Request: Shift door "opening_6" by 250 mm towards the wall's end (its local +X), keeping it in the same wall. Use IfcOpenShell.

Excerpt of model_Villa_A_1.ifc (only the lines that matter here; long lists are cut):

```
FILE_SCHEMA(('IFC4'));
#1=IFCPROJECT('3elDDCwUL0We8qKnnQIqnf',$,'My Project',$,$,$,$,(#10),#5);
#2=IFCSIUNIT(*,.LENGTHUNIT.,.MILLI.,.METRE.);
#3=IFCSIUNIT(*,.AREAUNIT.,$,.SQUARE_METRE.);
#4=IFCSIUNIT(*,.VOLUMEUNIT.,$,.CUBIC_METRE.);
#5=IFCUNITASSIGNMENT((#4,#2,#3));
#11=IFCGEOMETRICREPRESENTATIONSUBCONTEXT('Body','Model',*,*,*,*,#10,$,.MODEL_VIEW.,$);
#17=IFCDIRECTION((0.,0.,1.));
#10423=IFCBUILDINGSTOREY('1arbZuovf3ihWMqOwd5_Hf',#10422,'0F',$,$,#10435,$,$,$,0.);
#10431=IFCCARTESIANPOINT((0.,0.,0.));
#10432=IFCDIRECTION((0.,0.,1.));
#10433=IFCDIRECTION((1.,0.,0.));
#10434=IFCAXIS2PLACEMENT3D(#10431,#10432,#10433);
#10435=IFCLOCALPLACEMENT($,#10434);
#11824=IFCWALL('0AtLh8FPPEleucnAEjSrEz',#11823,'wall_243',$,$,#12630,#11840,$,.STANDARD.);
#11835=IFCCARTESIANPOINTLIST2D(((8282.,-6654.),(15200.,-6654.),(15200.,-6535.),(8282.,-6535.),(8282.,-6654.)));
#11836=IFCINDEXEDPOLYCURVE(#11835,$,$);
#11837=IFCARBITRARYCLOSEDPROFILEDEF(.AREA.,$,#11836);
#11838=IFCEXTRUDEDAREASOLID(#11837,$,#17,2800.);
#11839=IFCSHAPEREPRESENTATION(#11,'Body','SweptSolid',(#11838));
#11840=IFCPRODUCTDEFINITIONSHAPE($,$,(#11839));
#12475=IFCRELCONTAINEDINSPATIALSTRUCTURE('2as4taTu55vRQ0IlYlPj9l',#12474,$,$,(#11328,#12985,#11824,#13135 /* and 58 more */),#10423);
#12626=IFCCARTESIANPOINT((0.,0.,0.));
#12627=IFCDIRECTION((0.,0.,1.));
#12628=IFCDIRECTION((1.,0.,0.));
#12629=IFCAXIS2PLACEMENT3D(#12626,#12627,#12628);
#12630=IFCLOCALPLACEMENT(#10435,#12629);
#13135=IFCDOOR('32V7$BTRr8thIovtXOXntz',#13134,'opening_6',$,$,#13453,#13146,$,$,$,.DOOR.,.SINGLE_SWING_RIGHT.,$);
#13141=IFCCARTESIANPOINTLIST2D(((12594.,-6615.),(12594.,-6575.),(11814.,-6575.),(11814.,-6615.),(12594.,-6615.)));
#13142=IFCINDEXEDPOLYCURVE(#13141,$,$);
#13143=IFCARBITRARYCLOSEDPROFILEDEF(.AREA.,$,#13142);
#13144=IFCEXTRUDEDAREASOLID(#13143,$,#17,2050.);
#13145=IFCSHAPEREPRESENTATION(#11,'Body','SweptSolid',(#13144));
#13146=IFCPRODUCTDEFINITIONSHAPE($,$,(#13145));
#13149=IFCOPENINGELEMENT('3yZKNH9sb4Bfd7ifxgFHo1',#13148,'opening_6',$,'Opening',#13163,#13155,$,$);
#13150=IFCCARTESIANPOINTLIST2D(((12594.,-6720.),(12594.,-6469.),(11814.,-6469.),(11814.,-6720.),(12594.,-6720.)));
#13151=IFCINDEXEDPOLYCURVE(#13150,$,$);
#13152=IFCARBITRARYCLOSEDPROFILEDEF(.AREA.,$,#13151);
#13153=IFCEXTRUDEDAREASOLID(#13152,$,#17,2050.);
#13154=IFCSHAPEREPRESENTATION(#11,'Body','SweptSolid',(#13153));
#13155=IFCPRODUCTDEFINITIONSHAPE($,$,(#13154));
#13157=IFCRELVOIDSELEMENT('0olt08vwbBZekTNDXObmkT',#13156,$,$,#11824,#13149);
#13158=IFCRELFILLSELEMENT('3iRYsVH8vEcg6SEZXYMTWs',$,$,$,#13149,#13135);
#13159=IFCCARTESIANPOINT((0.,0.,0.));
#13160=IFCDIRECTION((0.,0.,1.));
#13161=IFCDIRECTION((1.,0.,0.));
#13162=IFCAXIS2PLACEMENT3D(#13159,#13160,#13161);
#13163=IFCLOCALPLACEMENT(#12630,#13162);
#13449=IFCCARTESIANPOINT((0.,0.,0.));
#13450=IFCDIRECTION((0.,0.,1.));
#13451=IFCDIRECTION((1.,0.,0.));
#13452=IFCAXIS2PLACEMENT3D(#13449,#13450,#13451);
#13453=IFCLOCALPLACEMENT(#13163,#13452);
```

```python
import ifcopenshell
import ifcopenshell.api.geometry
import ifcopenshell.util.placement
import ifcopenshell.util.unit

model = ifcopenshell.open("model_Villa_A_1.ifc")
unit_scale = ifcopenshell.util.unit.calculate_unit_scale(model)

door = model.by_guid("32V7$BTRr8thIovtXOXntz")
opening = door.FillsVoids[0].RelatingOpeningElement
wall = opening.VoidsElements[0].RelatingBuildingElement

wall_matrix = ifcopenshell.util.placement.get_local_placement(wall.ObjectPlacement)
shift = wall_matrix[:3, 0] * 0.25 / unit_scale
before = ifcopenshell.util.placement.get_local_placement(door.ObjectPlacement)[:3, 3].copy()

# The door is placed relative to its opening, so it follows when the opening moves.
matrix = ifcopenshell.util.placement.get_local_placement(opening.ObjectPlacement)
matrix[:3, 3] += shift
ifcopenshell.api.geometry.edit_object_placement(
    model, product=opening, matrix=matrix, is_si=False, should_transform_children=True
)

after = ifcopenshell.util.placement.get_local_placement(door.ObjectPlacement)[:3, 3]
print("door moved by", (after - before).round(3) + 0.0)

model.write("model_Villa_A_1_edited.ifc")
```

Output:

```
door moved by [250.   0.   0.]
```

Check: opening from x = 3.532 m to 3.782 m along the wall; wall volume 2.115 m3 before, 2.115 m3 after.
